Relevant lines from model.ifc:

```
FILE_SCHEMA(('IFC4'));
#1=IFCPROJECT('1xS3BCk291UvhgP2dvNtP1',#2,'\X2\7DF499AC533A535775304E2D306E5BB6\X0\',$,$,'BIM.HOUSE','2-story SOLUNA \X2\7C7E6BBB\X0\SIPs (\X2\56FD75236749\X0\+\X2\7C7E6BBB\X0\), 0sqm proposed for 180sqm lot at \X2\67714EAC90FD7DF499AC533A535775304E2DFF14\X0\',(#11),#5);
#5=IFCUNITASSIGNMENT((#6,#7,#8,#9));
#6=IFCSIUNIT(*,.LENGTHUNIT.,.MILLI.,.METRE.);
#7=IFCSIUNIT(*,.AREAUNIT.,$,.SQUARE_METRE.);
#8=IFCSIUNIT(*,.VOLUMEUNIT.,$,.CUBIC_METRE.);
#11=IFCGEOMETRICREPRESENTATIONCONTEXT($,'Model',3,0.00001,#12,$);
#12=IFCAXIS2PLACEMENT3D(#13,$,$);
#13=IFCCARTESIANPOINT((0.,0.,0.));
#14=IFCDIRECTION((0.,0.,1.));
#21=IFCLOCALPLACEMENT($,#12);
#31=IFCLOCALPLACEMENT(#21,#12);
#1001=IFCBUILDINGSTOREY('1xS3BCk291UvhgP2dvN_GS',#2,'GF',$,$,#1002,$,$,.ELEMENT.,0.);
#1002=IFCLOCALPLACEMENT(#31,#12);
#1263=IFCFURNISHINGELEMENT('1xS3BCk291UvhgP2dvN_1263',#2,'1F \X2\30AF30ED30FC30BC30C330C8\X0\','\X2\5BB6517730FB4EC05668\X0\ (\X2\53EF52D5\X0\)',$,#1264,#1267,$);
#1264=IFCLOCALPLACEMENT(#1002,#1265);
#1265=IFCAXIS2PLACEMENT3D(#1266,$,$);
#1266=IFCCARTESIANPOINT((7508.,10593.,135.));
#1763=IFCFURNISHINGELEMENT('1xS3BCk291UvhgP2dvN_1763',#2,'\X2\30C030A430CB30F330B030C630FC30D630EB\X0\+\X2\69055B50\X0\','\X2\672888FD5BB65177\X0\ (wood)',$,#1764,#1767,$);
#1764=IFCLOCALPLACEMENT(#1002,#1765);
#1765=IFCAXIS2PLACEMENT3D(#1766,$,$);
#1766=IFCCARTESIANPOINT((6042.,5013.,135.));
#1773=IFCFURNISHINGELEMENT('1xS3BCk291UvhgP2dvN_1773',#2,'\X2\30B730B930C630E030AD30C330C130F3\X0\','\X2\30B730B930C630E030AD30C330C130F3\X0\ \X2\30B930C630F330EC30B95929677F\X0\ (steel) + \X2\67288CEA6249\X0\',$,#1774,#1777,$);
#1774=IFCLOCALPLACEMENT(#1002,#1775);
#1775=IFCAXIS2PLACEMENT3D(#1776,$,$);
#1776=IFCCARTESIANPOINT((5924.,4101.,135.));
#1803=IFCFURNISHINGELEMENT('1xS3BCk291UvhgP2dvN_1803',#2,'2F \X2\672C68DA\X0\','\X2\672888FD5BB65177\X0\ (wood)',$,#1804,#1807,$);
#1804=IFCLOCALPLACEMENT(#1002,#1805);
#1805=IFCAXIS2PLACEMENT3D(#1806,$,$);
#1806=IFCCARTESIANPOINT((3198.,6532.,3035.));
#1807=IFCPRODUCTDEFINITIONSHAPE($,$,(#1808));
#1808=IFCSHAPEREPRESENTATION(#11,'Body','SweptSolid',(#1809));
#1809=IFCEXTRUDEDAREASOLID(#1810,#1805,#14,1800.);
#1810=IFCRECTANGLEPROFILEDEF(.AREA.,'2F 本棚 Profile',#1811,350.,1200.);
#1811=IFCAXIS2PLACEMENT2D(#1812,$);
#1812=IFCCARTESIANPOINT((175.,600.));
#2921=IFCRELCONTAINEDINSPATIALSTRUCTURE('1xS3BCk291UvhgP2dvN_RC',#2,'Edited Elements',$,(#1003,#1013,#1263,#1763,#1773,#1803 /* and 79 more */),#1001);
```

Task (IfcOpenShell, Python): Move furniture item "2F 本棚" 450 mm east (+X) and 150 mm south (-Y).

```python
import ifcopenshell
import ifcopenshell.api.geometry
import ifcopenshell.util.placement

model = ifcopenshell.open("model.ifc")

item = model.by_guid("1xS3BCk291UvhgP2dvN_1803")
matrix = ifcopenshell.util.placement.get_local_placement(item.ObjectPlacement)
matrix[0, 3] += 450.0
matrix[1, 3] -= 150.0
ifcopenshell.api.geometry.edit_object_placement(model, product=item, matrix=matrix, is_si=False)

print(ifcopenshell.util.placement.get_local_placement(item.ObjectPlacement).round(3) + 0.0)

model.write("model_v2.ifc")
```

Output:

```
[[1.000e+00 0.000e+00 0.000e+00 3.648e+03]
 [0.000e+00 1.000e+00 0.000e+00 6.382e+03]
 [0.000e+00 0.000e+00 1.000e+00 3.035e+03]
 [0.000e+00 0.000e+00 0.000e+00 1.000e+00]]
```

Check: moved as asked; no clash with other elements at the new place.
